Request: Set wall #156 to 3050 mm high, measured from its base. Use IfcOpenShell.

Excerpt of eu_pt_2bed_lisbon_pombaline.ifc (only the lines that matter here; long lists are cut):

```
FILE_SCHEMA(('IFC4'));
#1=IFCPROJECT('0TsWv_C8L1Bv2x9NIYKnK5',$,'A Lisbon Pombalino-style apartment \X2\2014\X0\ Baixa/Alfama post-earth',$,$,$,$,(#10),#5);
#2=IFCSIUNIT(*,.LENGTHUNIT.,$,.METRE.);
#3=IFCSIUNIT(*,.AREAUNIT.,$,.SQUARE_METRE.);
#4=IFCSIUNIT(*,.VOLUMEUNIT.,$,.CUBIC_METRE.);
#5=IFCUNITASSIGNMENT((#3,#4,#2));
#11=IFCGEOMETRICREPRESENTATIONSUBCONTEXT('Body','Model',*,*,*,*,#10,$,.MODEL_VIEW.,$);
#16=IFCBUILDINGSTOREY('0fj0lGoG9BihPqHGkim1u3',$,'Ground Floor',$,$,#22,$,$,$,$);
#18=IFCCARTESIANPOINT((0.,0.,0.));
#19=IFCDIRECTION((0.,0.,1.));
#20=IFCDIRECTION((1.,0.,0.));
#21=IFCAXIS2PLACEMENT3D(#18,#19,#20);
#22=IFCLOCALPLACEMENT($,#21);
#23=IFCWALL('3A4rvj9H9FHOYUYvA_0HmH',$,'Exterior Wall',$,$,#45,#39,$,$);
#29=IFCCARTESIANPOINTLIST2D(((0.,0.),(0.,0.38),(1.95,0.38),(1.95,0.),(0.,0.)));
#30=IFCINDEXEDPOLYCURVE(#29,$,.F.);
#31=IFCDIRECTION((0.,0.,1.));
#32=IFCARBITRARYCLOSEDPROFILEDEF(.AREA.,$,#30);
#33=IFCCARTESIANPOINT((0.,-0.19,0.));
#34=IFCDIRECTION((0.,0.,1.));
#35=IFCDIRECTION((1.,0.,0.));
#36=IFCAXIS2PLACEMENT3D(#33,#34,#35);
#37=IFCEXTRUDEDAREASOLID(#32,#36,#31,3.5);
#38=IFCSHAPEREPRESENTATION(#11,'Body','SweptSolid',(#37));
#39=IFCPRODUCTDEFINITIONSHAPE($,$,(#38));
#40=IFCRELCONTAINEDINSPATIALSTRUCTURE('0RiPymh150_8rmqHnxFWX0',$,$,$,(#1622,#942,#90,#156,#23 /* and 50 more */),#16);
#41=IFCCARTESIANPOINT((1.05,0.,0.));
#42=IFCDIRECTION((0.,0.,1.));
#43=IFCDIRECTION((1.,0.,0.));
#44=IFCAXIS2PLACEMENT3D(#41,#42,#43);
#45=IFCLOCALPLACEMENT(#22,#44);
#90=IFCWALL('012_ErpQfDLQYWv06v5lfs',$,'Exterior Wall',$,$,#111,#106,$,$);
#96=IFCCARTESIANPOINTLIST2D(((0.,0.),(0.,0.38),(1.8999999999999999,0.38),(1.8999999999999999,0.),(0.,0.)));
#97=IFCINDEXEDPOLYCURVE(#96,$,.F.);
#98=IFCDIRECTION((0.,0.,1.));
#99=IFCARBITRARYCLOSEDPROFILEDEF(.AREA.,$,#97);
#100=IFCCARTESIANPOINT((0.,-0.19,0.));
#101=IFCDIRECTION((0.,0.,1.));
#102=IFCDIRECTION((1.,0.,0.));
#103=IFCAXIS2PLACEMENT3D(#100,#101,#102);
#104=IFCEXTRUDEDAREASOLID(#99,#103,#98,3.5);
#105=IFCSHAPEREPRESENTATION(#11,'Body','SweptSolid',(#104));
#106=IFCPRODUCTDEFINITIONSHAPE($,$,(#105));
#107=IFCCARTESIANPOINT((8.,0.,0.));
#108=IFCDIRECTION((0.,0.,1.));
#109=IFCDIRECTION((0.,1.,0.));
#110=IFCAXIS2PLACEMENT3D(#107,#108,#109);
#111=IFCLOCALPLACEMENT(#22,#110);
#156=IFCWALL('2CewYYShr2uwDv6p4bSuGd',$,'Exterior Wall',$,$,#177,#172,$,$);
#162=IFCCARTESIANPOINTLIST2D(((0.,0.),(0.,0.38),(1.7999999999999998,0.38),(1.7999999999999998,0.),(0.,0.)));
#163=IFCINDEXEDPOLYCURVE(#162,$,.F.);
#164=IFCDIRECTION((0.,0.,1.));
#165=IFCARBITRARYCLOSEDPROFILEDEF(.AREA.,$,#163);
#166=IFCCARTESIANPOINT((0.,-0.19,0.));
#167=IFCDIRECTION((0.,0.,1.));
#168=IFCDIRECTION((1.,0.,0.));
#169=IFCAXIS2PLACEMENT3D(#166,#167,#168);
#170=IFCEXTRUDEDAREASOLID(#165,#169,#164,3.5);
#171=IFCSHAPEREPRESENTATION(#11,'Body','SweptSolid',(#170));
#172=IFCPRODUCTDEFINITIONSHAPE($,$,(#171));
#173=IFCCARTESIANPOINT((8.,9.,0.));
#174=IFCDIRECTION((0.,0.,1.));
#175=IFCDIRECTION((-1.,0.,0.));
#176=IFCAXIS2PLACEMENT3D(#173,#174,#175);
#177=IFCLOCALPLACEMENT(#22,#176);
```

```python
import ifcopenshell
import ifcopenshell.geom
import ifcopenshell.util.representation
import ifcopenshell.util.shape

model = ifcopenshell.open("eu_pt_2bed_lisbon_pombaline.ifc")
settings = ifcopenshell.geom.settings()


def volume(element):
    """Net volume in cubic metres, openings subtracted."""
    shape = ifcopenshell.geom.create_shape(settings, element)
    return ifcopenshell.util.shape.get_volume(shape.geometry)


wall = model.by_id(156)
before = volume(wall)

body = ifcopenshell.util.representation.get_representation(wall, "Model", "Body")
solid = body.Items[0]
old_height = solid.Depth
solid.Depth = 3.05
after = volume(wall)

print(f"height {old_height:g} -> {solid.Depth:g}, volume {before:.3f} -> {after:.3f} m3")

model.write("eu_pt_2bed_lisbon_pombaline_updated.ifc")
```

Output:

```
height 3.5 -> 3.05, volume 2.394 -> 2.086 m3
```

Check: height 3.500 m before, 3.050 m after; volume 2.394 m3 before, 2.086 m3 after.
